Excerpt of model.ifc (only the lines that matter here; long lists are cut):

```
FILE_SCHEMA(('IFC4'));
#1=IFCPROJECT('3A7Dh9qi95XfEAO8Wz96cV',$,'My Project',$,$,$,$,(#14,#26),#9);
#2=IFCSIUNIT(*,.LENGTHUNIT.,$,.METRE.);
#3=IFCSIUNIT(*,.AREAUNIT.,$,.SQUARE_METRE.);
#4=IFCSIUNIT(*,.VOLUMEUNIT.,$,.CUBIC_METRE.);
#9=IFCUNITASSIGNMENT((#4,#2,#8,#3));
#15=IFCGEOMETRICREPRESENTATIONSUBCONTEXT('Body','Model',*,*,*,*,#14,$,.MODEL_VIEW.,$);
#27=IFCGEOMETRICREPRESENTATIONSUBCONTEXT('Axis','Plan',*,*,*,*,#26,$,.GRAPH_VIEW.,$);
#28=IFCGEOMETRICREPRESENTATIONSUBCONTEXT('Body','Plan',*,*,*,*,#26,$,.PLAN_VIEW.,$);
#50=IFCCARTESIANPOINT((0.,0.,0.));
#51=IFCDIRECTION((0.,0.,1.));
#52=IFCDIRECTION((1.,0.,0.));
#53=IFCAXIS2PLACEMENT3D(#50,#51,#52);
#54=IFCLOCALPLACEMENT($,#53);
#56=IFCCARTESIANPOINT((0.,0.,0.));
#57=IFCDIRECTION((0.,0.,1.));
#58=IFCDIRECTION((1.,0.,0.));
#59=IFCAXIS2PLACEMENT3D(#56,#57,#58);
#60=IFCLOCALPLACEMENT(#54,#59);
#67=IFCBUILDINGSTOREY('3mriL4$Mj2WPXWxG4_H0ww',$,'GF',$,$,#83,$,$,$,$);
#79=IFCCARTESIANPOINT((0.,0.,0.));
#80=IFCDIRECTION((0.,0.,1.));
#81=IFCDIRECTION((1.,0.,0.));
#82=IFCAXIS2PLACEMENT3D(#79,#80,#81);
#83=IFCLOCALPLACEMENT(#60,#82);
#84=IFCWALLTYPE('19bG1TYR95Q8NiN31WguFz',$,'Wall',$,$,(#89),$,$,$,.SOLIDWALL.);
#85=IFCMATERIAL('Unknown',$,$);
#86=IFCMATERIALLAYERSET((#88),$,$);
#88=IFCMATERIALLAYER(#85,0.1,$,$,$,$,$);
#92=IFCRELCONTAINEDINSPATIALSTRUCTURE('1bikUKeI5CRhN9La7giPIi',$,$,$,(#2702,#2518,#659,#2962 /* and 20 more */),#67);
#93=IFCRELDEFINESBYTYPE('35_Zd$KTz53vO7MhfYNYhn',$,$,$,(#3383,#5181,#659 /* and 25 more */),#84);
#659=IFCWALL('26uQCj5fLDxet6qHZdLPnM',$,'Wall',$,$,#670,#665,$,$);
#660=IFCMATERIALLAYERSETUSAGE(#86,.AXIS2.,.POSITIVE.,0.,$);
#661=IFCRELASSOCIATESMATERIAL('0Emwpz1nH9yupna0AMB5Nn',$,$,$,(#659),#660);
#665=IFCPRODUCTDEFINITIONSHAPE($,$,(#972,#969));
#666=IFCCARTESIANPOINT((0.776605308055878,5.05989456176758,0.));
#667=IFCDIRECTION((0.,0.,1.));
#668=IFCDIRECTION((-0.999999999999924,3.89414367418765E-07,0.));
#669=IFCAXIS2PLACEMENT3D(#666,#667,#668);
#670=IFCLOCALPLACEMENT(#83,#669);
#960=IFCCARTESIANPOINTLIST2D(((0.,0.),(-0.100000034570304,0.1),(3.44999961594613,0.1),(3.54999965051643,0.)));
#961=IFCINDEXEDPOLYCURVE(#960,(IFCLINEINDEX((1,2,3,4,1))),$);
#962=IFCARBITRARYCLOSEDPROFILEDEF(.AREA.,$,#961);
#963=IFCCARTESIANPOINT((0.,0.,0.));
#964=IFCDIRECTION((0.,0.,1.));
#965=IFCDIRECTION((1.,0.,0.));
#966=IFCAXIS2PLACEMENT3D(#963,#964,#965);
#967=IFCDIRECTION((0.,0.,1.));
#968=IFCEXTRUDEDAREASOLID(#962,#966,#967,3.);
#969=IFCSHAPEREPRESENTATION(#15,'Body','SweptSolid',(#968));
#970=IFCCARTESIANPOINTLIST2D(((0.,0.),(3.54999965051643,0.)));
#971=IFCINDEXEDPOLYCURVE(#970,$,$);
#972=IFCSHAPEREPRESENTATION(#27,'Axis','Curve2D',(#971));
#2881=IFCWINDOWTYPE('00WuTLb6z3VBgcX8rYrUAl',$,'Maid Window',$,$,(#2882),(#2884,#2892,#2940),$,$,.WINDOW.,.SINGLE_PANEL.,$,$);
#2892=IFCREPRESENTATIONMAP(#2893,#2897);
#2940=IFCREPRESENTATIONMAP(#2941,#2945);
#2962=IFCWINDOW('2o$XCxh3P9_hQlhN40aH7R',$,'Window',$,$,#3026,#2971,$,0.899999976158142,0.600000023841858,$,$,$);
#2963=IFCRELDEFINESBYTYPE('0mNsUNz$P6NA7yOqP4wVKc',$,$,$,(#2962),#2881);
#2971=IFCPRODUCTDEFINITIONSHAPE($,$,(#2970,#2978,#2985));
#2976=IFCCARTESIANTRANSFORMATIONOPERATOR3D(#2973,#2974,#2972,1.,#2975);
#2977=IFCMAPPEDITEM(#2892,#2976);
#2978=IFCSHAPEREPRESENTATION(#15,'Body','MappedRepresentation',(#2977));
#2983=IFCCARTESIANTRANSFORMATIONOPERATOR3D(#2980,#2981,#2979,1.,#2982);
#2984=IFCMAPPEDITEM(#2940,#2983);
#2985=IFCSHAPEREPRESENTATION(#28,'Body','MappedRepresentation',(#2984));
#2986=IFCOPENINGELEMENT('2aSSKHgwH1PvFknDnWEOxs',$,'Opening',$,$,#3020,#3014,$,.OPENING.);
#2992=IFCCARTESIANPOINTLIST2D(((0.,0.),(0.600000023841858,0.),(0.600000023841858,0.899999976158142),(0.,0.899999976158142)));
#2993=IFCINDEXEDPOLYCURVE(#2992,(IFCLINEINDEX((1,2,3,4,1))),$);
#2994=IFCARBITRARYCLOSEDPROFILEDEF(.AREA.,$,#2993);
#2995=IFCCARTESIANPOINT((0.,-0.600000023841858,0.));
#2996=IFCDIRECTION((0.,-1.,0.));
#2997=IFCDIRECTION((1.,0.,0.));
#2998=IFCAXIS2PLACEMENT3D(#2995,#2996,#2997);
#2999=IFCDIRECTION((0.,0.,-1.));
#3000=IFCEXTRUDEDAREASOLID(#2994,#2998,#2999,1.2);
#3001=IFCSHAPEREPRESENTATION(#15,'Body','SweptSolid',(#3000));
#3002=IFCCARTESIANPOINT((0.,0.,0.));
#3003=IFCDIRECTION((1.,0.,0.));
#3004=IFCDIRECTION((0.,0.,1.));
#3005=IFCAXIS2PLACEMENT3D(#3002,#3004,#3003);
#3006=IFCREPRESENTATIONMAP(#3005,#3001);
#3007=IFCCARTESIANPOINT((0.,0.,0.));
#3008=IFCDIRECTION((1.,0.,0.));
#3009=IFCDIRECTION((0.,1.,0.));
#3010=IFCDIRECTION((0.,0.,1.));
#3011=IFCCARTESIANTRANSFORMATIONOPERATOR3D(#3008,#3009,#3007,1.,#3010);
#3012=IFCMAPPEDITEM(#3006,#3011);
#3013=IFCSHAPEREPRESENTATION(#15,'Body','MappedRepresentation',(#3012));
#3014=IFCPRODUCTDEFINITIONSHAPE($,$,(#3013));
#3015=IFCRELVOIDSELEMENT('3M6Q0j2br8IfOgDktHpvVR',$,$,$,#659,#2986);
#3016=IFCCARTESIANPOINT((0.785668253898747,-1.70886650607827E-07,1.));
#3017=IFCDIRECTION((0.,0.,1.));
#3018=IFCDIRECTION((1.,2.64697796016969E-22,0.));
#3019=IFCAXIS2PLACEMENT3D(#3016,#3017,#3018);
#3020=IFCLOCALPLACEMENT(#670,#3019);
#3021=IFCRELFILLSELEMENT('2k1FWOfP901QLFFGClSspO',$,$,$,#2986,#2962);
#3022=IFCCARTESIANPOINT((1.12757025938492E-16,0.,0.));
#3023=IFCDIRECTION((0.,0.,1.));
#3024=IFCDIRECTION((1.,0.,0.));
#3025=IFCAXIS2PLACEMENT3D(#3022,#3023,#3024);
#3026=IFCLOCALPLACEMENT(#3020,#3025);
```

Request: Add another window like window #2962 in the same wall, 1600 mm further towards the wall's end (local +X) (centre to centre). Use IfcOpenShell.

```python
import ifcopenshell
import ifcopenshell.api.feature
import ifcopenshell.api.geometry
import ifcopenshell.api.root
import ifcopenshell.geom
import ifcopenshell.util.element
import ifcopenshell.util.placement
import ifcopenshell.util.shape

model = ifcopenshell.open("model.ifc")
settings = ifcopenshell.geom.settings()


def volume(element):
    """Net volume in cubic metres, openings subtracted."""
    shape = ifcopenshell.geom.create_shape(settings, element)
    return ifcopenshell.util.shape.get_volume(shape.geometry)


window = model.by_guid("2o$XCxh3P9_hQlhN40aH7R")
opening = window.FillsVoids[0].RelatingOpeningElement
wall = opening.VoidsElements[0].RelatingBuildingElement
before = volume(wall)
shift = ifcopenshell.util.placement.get_local_placement(wall.ObjectPlacement)[:3, 0] * 1.6

# copy_class copies the void relationship, type, container and properties, but no geometry.
new_opening = ifcopenshell.api.root.copy_class(model, product=opening)
new_opening.Representation = ifcopenshell.util.element.copy_deep(
    model, opening.Representation, exclude=["IfcGeometricRepresentationContext", "IfcRepresentationMap"]
)
new_window = ifcopenshell.api.root.copy_class(model, product=window)
new_window.Representation = ifcopenshell.util.element.copy_deep(
    model, window.Representation, exclude=["IfcGeometricRepresentationContext", "IfcRepresentationMap"]
)
ifcopenshell.api.feature.add_filling(model, opening=new_opening, element=new_window)

for old, new in ((opening, new_opening), (window, new_window)):
    matrix = ifcopenshell.util.placement.get_local_placement(old.ObjectPlacement)
    matrix[:3, 3] += shift
    ifcopenshell.api.geometry.edit_object_placement(model, product=new, matrix=matrix, is_si=False)

after = volume(wall)

print(f"wall volume {before:.3f} -> {after:.3f} m3")

model.write("model_updated.ifc")
```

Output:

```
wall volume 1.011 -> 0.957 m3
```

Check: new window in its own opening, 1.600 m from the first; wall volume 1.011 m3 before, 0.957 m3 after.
